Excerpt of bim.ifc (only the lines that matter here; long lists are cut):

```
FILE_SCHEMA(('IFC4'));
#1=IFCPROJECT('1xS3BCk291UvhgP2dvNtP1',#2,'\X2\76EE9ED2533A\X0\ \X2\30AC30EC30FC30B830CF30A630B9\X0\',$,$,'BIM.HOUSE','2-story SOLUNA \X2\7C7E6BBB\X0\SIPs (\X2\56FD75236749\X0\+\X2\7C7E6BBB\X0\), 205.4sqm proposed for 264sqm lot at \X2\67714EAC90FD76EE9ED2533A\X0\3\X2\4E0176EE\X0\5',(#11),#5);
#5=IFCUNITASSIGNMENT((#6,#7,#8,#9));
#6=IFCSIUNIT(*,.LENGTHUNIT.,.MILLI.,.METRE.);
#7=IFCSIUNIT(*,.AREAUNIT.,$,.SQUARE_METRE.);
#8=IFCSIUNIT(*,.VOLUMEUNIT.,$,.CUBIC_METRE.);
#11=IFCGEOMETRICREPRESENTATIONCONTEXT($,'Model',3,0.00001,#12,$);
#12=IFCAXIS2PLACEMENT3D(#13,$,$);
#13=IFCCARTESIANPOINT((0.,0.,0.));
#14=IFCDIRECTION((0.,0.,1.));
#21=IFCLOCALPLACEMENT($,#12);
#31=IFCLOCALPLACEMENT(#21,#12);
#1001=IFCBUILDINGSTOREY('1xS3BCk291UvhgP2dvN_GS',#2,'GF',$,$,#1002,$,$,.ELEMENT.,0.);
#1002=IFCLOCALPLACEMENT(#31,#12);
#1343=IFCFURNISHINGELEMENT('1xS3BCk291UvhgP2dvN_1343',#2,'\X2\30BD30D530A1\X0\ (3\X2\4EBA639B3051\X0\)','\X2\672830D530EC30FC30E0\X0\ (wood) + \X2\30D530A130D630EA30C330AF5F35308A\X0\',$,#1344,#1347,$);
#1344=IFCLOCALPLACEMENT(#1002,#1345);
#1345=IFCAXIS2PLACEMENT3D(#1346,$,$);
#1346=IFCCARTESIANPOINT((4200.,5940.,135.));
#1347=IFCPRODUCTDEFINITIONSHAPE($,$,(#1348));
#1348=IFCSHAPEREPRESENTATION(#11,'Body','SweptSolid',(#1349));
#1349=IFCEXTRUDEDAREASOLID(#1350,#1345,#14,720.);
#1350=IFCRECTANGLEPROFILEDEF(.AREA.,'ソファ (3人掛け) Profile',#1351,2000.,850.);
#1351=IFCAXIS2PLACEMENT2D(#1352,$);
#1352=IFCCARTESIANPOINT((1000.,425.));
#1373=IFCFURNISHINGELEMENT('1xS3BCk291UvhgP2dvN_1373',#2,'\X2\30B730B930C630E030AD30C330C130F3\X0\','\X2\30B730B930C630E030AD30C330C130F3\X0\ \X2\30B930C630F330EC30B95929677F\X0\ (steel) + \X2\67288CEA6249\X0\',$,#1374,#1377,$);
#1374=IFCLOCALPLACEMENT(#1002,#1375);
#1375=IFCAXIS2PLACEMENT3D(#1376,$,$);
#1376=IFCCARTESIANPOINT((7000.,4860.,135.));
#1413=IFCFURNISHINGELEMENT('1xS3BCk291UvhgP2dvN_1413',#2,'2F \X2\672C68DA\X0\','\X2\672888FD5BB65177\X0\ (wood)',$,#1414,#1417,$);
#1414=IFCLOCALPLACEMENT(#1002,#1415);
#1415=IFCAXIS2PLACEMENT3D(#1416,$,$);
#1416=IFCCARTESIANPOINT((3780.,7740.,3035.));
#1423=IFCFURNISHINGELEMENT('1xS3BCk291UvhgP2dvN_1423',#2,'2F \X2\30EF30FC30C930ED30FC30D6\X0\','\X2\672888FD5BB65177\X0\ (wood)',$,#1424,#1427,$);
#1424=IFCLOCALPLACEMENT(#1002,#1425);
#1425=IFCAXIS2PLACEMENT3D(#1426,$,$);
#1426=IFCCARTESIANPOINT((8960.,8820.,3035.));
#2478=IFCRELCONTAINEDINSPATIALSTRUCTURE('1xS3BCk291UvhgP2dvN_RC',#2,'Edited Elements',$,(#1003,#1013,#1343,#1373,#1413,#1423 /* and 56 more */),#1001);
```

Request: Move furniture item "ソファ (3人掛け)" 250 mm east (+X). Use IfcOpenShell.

```python
import ifcopenshell
import ifcopenshell.api.geometry
import ifcopenshell.util.placement
import ifcopenshell.util.unit

model = ifcopenshell.open("bim.ifc")
unit_scale = ifcopenshell.util.unit.calculate_unit_scale(model)

item = model.by_guid("1xS3BCk291UvhgP2dvN_1343")
matrix = ifcopenshell.util.placement.get_local_placement(item.ObjectPlacement)
matrix[0, 3] += 0.25 / unit_scale
ifcopenshell.api.geometry.edit_object_placement(model, product=item, matrix=matrix, is_si=False)

print(ifcopenshell.util.placement.get_local_placement(item.ObjectPlacement).round(3) + 0.0)

model.write("bim-out.ifc")
```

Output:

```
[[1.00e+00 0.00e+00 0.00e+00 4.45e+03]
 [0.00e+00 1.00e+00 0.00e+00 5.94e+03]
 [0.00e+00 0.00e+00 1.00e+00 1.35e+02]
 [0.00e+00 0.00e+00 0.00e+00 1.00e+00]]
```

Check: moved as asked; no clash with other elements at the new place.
